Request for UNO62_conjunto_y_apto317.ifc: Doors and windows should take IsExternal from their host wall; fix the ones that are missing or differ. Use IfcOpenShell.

First a look at what the model holds.

```python
import ifcopenshell
import ifcopenshell.util.element

model = ifcopenshell.open("UNO62_conjunto_y_apto317.ifc")
print(model.schema)
seen = {}
for e in model.by_type("IfcDoor") + model.by_type("IfcWindow"):
    if not e.FillsVoids:
        continue
    host = e.FillsVoids[0].RelatingOpeningElement.VoidsElements[0].RelatingBuildingElement
    own = ifcopenshell.util.element.get_pset(e, f"Pset_{e.is_a()[3:].removesuffix('StandardCase')}Common", "IsExternal")
    wall = ifcopenshell.util.element.get_pset(host, "Pset_WallCommon", "IsExternal")
    seen[e.is_a(), own, wall] = seen.get((e.is_a(), own, wall), 0) + 1
for (cls, own, wall), count in sorted(seen.items(), key=str):
    print(count, cls, "IsExternal:", own, "| host wall:", wall)
```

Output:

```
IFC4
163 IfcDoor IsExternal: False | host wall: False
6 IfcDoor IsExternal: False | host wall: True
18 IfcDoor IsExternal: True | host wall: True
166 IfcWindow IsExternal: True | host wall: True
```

```python
import ifcopenshell
import ifcopenshell.api.pset
import ifcopenshell.util.element

model = ifcopenshell.open("UNO62_conjunto_y_apto317.ifc")

count = 0
for ifc_class, pset_name in (("IfcDoor", "Pset_DoorCommon"), ("IfcWindow", "Pset_WindowCommon")):
    for e in model.by_type(ifc_class):
        if not e.FillsVoids:
            continue
        host = e.FillsVoids[0].RelatingOpeningElement.VoidsElements[0].RelatingBuildingElement
        external = ifcopenshell.util.element.get_pset(host, "Pset_WallCommon", "IsExternal")
        if external is None or ifcopenshell.util.element.get_pset(e, pset_name, "IsExternal") == external:
            continue
        found = ifcopenshell.util.element.get_pset(e, pset_name, should_inherit=False)
        if found:
            pset = model.by_id(found["id"])
            if len(ifcopenshell.util.element.get_elements_by_pset(pset)) > 1:
                pset = ifcopenshell.api.pset.unshare_pset(model, products=[e], pset=pset)[0]
        else:
            pset = ifcopenshell.api.pset.add_pset(model, product=e, name=pset_name)
        ifcopenshell.api.pset.edit_pset(model, pset=pset, properties={"IsExternal": external})
        count += 1

print(count, "updated")

model.write("UNO62_conjunto_y_apto317_v2.ifc")
```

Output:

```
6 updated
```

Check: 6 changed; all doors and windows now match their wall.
